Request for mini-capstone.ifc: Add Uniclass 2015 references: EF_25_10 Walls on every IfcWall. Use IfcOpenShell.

First a look at what the model holds.

```python
import ifcopenshell

model = ifcopenshell.open("mini-capstone.ifc")
print(model.schema)
print("classifications:", [c.Name for c in model.by_type("IfcClassification")])
for ifc_class in ("IfcDoor", "IfcRoof", "IfcStair", "IfcWall", "IfcWindow"):
    print(ifc_class, len(model.by_type(ifc_class)))
```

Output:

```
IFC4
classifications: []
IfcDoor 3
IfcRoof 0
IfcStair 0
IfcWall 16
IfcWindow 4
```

```python
import ifcopenshell
import ifcopenshell.api.classification

model = ifcopenshell.open("mini-capstone.ifc")

system = ifcopenshell.api.classification.add_classification(model, classification="Uniclass 2015")

codes = {
    "IfcWall": ("EF_25_10", "Walls"),
}
for ifc_class, (code, name) in codes.items():
    products = model.by_type(ifc_class)
    ifcopenshell.api.classification.add_reference(
        model, products=products, classification=system, identification=code, name=name
    )
    print(code, len(products))

model.write("mini-capstone_rev.ifc")
```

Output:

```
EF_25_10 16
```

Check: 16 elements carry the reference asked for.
